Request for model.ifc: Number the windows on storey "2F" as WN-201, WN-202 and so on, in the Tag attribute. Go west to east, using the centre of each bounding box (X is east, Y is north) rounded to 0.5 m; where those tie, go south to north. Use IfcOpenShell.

First a look at what the model holds.

```python
import ifcopenshell
import ifcopenshell.util.element
import ifcopenshell.util.placement

model = ifcopenshell.open("model.ifc")
print(model.schema)
storey = next(s for s in model.by_type("IfcBuildingStorey") if s.Name == "2F")
windows = [e for e in ifcopenshell.util.element.get_decomposition(storey) if e.is_a("IfcWindow")]
for e in sorted(windows, key=lambda e: e.id()):
    origin = ifcopenshell.util.placement.get_local_placement(e.ObjectPlacement)[:3, 3]
    print(e.id(), e.Tag, e.Name, origin.round(2) + 0.0, sep=" | ")
```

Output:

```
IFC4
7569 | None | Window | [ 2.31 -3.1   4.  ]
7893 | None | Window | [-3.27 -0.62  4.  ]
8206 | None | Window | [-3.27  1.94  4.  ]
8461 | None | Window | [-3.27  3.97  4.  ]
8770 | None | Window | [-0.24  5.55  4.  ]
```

```python
import ifcopenshell
import ifcopenshell.geom
import ifcopenshell.util.element
import ifcopenshell.util.shape

model = ifcopenshell.open("model.ifc")
settings = ifcopenshell.geom.settings()
settings.set("use-world-coords", True)


def centre(element):
    shape = ifcopenshell.geom.create_shape(settings, element)
    return ifcopenshell.util.shape.get_bbox_centroid(shape.geometry)


storey = next(s for s in model.by_type("IfcBuildingStorey") if s.Name == "2F")
windows = [e for e in ifcopenshell.util.element.get_decomposition(storey) if e.is_a("IfcWindow")]

# Insertion points can sit at a corner or the storey origin, so sort by the geometry (in metres).
centres = {e: centre(e) for e in windows}
windows.sort(key=lambda e: (round(centres[e][0] / 0.5), centres[e][1]))

for i, e in enumerate(windows, start=1):
    number = f"WN-2{i:02d}"
    e.Tag = number
    print(e.id(), number)

model.write("model_v2.ifc")
```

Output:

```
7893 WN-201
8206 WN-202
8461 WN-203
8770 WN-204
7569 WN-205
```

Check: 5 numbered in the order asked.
